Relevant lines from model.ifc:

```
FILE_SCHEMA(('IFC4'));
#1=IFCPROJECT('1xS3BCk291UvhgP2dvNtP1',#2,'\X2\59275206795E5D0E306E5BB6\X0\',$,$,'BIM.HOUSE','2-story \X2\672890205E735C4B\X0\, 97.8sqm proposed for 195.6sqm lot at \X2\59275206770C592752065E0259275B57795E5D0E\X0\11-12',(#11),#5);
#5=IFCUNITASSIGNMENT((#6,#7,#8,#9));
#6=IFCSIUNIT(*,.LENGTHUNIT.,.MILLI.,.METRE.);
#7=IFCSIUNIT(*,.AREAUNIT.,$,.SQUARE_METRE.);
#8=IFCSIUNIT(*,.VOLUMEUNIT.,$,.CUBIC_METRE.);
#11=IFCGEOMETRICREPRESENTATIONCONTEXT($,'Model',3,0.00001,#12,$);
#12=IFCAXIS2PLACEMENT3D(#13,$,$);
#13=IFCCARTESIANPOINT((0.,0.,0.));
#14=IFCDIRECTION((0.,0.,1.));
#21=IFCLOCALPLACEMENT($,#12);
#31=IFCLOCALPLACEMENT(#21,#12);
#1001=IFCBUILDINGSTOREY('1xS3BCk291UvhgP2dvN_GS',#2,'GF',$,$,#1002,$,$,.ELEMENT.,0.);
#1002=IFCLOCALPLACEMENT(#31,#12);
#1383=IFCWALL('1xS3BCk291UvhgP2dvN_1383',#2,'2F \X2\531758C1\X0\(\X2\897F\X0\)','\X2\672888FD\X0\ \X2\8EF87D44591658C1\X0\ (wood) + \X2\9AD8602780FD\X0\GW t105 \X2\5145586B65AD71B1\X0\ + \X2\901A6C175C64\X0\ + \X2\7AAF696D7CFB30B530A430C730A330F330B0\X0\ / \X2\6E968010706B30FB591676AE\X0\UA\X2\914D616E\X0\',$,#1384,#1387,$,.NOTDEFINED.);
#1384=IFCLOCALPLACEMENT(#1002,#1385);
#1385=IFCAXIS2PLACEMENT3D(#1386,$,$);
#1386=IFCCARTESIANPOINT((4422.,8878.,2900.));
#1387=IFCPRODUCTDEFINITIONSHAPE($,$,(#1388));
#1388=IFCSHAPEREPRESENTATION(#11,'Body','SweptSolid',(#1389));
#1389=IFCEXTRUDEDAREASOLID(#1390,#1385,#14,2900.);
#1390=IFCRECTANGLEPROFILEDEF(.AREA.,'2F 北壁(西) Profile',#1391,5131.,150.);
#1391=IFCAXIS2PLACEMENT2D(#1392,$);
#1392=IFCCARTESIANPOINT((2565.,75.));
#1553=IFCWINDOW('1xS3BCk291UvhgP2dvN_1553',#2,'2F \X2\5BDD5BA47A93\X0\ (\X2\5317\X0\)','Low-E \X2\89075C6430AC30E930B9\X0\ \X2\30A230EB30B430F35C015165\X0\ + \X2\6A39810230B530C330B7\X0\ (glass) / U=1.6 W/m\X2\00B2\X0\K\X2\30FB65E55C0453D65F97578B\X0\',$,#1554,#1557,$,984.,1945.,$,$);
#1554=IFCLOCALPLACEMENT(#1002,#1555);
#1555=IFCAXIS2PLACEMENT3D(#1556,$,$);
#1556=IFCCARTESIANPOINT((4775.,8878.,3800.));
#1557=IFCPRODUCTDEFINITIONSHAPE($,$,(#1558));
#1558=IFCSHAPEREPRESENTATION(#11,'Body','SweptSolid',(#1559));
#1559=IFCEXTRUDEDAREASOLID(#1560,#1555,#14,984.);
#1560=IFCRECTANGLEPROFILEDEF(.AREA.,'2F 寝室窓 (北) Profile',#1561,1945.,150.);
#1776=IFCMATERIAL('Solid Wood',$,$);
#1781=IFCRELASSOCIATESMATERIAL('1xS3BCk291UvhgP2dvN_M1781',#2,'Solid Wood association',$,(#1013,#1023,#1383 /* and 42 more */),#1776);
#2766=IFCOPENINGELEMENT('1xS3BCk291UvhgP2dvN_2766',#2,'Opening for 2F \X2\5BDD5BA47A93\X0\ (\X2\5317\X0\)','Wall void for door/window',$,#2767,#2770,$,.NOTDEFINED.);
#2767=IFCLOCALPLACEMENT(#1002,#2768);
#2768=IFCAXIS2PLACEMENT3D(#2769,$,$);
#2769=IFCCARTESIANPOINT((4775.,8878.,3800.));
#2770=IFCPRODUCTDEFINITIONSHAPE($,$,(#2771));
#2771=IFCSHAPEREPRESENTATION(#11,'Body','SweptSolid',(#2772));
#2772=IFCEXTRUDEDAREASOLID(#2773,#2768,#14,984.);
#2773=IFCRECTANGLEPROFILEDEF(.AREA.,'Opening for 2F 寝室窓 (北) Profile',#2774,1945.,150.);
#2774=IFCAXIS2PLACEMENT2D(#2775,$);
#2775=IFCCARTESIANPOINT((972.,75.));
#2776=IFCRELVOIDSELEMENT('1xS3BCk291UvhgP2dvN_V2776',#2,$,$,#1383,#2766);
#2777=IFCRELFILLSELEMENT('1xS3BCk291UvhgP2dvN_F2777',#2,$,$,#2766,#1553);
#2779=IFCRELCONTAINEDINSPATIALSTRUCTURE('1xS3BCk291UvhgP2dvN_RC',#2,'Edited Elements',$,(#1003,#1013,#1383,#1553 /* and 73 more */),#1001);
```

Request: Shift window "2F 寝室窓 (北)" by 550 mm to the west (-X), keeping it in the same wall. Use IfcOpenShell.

```python
import ifcopenshell
import ifcopenshell.api.geometry
import ifcopenshell.util.placement

model = ifcopenshell.open("model.ifc")

window = model.by_id(1553)
opening = window.FillsVoids[0].RelatingOpeningElement
wall = opening.VoidsElements[0].RelatingBuildingElement

wall_matrix = ifcopenshell.util.placement.get_local_placement(wall.ObjectPlacement)
shift = wall_matrix[:3, 0] * -550.0
before = ifcopenshell.util.placement.get_local_placement(window.ObjectPlacement)[:3, 3].copy()

# The window is not placed relative to its opening, so move both.
for product in (opening, window):
    matrix = ifcopenshell.util.placement.get_local_placement(product.ObjectPlacement)
    matrix[:3, 3] += shift
    ifcopenshell.api.geometry.edit_object_placement(model, product=product, matrix=matrix, is_si=False)

after = ifcopenshell.util.placement.get_local_placement(window.ObjectPlacement)[:3, 3]
print("window moved by", (after - before).round(3) + 0.0)

model.write("model-out.ifc")
```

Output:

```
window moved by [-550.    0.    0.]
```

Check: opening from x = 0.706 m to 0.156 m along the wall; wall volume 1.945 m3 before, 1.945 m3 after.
